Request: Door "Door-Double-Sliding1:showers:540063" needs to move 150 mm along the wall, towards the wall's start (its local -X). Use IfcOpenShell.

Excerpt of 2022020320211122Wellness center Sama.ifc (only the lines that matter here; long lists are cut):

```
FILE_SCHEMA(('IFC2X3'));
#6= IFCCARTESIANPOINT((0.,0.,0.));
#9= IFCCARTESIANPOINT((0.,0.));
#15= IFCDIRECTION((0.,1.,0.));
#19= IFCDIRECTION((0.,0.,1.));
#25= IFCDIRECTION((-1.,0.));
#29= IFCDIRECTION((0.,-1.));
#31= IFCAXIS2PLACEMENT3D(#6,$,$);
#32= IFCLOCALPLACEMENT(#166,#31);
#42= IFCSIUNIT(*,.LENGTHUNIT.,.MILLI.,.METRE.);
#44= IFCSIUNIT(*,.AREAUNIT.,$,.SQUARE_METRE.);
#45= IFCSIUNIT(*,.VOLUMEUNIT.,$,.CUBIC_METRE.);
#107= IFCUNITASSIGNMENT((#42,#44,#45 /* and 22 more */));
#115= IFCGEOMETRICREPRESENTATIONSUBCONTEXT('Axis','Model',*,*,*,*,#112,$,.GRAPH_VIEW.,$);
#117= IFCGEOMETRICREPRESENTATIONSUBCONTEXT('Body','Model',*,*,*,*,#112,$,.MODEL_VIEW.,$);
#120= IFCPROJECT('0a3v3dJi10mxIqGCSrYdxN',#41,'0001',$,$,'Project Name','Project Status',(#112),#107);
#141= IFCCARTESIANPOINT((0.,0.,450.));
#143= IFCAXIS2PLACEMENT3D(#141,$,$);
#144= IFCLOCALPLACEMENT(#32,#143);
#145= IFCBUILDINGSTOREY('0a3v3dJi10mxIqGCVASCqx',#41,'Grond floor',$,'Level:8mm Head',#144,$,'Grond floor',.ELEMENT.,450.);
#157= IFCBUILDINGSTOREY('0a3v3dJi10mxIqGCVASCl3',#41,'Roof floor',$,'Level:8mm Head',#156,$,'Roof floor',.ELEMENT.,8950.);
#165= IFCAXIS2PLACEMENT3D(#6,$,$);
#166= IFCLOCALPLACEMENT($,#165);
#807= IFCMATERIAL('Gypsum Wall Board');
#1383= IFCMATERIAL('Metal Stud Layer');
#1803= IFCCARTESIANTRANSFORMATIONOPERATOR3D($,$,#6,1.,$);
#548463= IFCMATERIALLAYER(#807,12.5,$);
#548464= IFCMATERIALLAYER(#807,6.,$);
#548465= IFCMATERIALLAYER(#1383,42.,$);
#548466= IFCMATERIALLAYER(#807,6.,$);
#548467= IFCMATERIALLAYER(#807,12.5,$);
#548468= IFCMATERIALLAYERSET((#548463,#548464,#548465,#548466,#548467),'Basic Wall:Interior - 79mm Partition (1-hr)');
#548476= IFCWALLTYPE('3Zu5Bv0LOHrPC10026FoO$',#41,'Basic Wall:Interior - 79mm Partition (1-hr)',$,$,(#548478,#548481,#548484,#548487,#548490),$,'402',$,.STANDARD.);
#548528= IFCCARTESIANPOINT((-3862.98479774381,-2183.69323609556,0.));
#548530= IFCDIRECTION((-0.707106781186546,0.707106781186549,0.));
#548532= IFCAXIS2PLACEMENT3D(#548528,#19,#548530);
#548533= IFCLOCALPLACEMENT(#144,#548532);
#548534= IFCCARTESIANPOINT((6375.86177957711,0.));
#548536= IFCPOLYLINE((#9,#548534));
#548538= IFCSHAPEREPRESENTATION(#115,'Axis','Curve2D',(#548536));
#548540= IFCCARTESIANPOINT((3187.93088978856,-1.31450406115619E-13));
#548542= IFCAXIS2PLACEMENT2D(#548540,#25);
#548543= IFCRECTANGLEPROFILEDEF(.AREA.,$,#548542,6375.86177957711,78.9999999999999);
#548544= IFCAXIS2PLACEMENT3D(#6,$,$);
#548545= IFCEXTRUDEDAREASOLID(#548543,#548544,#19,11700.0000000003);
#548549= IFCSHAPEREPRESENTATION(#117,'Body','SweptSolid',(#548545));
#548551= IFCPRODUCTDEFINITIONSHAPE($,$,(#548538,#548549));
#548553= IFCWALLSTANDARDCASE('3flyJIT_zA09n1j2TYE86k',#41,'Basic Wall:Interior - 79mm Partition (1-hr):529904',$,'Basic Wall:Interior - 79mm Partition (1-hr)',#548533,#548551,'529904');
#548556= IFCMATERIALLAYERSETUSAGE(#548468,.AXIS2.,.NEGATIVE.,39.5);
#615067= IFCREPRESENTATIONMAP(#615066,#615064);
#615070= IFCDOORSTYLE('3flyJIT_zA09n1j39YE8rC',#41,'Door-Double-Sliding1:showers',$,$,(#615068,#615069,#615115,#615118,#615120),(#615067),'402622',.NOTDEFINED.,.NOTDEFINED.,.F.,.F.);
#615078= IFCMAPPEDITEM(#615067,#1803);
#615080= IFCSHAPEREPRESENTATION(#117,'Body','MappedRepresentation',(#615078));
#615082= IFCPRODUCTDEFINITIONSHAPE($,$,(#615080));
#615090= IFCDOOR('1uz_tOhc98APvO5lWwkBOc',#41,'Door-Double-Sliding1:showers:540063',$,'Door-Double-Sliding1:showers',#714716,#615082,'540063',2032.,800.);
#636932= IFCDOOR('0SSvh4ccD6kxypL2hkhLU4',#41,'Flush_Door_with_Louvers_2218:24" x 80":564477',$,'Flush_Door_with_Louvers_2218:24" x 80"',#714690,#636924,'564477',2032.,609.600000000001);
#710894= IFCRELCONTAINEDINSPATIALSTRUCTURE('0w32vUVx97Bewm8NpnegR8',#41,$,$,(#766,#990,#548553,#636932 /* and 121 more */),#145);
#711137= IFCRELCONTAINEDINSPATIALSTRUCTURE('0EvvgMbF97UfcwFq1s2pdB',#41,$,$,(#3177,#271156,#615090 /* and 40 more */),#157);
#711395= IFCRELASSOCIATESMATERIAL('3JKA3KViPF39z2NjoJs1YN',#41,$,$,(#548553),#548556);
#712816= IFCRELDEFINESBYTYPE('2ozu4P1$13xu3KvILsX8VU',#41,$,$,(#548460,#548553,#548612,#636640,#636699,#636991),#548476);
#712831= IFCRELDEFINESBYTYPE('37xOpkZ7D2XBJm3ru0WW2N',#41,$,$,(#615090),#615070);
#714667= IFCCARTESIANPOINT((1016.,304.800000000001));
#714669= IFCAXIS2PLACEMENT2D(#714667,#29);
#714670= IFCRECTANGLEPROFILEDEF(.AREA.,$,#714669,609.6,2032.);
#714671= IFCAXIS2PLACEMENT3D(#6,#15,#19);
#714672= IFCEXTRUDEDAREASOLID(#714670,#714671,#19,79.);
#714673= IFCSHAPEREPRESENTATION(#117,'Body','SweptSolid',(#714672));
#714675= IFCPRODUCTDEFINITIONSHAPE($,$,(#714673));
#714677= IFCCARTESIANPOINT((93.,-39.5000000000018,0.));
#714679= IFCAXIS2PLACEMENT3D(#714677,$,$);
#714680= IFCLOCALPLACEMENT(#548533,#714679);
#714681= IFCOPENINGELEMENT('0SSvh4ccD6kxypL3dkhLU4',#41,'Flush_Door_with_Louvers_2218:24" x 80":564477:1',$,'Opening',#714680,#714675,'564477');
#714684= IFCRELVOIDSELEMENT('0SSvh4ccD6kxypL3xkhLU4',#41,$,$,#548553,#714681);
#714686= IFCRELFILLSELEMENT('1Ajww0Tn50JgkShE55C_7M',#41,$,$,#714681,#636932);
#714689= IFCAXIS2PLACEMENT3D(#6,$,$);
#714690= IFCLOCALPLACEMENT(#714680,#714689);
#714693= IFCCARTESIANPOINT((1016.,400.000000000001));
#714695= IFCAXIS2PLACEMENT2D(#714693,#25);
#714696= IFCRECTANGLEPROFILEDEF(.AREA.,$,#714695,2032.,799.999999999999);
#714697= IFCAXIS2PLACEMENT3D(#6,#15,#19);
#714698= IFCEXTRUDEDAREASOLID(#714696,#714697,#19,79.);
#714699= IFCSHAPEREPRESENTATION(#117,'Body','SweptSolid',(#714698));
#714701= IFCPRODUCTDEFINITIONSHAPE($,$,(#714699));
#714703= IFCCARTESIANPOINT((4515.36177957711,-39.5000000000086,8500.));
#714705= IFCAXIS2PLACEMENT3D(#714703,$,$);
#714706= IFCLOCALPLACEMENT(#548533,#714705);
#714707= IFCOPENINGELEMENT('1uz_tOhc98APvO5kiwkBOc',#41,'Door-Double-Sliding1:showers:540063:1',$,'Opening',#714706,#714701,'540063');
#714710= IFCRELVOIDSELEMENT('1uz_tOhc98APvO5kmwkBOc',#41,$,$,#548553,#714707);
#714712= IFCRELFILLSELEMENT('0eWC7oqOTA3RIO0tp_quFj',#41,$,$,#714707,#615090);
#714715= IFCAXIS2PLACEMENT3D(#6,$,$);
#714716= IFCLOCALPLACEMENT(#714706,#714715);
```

```python
import ifcopenshell
import ifcopenshell.api.geometry
import ifcopenshell.util.placement
import ifcopenshell.util.unit

model = ifcopenshell.open("2022020320211122Wellness center Sama.ifc")
unit_scale = ifcopenshell.util.unit.calculate_unit_scale(model)

door = model.by_guid("1uz_tOhc98APvO5lWwkBOc")
opening = door.FillsVoids[0].RelatingOpeningElement
wall = opening.VoidsElements[0].RelatingBuildingElement

wall_matrix = ifcopenshell.util.placement.get_local_placement(wall.ObjectPlacement)
shift = wall_matrix[:3, 0] * -0.15 / unit_scale
before = ifcopenshell.util.placement.get_local_placement(door.ObjectPlacement)[:3, 3].copy()

# The door is placed relative to its opening, so it follows when the opening moves.
matrix = ifcopenshell.util.placement.get_local_placement(opening.ObjectPlacement)
matrix[:3, 3] += shift
ifcopenshell.api.geometry.edit_object_placement(
    model, product=opening, matrix=matrix, is_si=False, should_transform_children=True
)

after = ifcopenshell.util.placement.get_local_placement(door.ObjectPlacement)[:3, 3]
print("door moved by", (after - before).round(3) + 0.0)

model.write("2022020320211122Wellness center Sama_rev.ifc")
```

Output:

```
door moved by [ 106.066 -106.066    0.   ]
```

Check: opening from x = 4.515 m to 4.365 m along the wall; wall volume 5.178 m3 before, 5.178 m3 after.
